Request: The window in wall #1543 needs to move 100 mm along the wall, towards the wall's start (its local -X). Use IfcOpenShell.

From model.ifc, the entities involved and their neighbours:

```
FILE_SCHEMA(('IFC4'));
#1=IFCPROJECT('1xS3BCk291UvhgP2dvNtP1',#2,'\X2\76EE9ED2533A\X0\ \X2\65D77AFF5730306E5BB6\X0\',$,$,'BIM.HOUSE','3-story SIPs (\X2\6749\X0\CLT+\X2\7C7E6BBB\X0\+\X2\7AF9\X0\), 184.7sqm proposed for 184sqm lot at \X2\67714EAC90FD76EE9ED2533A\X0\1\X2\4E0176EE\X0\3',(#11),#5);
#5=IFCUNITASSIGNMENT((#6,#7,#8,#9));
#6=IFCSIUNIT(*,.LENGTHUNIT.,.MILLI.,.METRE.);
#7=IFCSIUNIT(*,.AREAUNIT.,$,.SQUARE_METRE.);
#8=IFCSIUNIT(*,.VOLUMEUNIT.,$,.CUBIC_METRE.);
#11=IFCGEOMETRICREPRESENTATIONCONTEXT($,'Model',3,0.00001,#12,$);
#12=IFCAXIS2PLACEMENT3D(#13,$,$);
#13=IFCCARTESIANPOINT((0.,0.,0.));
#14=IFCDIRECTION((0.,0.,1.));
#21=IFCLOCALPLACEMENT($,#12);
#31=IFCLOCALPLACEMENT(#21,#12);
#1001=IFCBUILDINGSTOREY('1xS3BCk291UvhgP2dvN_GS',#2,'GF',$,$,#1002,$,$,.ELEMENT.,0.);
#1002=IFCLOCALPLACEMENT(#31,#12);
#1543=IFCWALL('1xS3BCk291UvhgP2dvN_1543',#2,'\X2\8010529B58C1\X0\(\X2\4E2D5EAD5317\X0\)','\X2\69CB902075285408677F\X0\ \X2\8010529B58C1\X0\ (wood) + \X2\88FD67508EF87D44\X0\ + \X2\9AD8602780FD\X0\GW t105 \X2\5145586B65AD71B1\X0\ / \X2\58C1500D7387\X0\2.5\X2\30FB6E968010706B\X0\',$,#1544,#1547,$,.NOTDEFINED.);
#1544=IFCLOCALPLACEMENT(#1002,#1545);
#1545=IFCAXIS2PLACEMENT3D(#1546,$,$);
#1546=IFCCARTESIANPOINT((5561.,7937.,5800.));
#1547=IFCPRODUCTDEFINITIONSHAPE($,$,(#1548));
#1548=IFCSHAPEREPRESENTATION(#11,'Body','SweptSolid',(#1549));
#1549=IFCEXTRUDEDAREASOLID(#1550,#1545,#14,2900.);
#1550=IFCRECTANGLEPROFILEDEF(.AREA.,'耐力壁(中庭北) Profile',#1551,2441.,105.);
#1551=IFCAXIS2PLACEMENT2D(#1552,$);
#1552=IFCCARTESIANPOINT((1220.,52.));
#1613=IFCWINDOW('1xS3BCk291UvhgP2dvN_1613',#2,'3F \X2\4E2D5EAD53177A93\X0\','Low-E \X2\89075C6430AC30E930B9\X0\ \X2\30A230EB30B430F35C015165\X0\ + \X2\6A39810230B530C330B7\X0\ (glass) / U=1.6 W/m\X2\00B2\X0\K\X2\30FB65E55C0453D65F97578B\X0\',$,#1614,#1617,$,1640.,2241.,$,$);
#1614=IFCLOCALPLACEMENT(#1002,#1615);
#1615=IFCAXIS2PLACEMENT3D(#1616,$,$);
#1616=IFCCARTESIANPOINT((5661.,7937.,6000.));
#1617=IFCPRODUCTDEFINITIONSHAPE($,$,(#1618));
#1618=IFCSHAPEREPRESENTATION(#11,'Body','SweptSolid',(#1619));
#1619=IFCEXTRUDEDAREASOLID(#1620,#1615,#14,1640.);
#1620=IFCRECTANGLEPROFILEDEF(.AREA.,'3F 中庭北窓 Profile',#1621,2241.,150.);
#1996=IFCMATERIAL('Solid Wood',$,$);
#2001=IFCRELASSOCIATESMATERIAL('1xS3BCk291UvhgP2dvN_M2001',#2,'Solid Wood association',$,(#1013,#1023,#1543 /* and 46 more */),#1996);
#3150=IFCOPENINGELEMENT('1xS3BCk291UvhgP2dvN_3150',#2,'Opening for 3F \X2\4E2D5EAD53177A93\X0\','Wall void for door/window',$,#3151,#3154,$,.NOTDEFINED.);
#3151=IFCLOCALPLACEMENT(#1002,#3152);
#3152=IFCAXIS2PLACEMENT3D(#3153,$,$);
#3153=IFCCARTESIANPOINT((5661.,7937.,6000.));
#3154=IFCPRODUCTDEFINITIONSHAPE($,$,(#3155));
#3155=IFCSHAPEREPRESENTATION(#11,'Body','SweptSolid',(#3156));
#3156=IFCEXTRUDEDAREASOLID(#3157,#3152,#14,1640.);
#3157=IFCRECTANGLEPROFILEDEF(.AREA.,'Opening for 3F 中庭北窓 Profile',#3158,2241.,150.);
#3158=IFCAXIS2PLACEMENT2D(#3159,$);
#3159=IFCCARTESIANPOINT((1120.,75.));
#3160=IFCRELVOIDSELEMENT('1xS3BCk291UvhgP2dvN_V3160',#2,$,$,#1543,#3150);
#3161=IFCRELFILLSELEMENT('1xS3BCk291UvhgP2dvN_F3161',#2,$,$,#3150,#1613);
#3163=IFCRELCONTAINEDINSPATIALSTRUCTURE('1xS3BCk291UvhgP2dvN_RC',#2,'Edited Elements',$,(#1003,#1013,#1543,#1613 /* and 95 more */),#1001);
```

```python
import ifcopenshell
import ifcopenshell.api.geometry
import ifcopenshell.util.placement

model = ifcopenshell.open("model.ifc")

window = model.by_guid("1xS3BCk291UvhgP2dvN_1613")
opening = window.FillsVoids[0].RelatingOpeningElement
wall = opening.VoidsElements[0].RelatingBuildingElement

wall_matrix = ifcopenshell.util.placement.get_local_placement(wall.ObjectPlacement)
shift = wall_matrix[:3, 0] * -100.0
before = ifcopenshell.util.placement.get_local_placement(window.ObjectPlacement)[:3, 3].copy()

# The window is not placed relative to its opening, so move both.
for product in (opening, window):
    matrix = ifcopenshell.util.placement.get_local_placement(product.ObjectPlacement)
    matrix[:3, 3] += shift
    ifcopenshell.api.geometry.edit_object_placement(model, product=product, matrix=matrix, is_si=False)

after = ifcopenshell.util.placement.get_local_placement(window.ObjectPlacement)[:3, 3]
print("window moved by", (after - before).round(3) + 0.0)

model.write("model_v2.ifc")
```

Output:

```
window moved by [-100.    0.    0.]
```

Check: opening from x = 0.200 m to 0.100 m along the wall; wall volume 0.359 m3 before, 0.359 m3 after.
